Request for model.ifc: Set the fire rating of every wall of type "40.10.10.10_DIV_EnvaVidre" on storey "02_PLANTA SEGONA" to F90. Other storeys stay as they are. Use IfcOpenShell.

First a look at what the model holds.

```python
import ifcopenshell
import ifcopenshell.util.element

model = ifcopenshell.open("model.ifc")
print(model.schema)
storey = next(s for s in model.by_type("IfcBuildingStorey") if s.Name == "02_PLANTA SEGONA")
walls = [e for e in ifcopenshell.util.element.get_decomposition(storey) if e.is_a("IfcWall")]
seen = {}
for e in walls:
    element_type = ifcopenshell.util.element.get_type(e)
    key = (element_type.Name if element_type != e and element_type else None, ifcopenshell.util.element.get_pset(e, "Pset_WallCommon", "FireRating"))
    seen[key] = seen.get(key, 0) + 1
for (name, value), count in sorted(seen.items(), key=str):
    print(count, "x", name, "|", value)
```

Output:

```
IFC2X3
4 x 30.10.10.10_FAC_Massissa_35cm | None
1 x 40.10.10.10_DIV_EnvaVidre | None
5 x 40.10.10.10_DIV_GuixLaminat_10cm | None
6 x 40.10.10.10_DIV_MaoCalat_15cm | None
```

```python
import ifcopenshell
import ifcopenshell.api.pset
import ifcopenshell.util.element

model = ifcopenshell.open("model.ifc")

storey = next(s for s in model.by_type("IfcBuildingStorey") if s.Name == "02_PLANTA SEGONA")
walls = [e for e in ifcopenshell.util.element.get_decomposition(storey) if e.is_a("IfcWall")]

count = 0
for e in walls:
    element_type = ifcopenshell.util.element.get_type(e)
    if element_type in (None, e) or element_type.Name != "40.10.10.10_DIV_EnvaVidre":
        continue
    # add_pset returns the element's existing set when there is one.
    pset = ifcopenshell.api.pset.add_pset(model, product=e, name="Pset_WallCommon")
    ifcopenshell.api.pset.edit_pset(model, pset=pset, properties={"FireRating": "F90"})
    count += 1

print(count, "walls updated")

model.write("model-out.ifc")
```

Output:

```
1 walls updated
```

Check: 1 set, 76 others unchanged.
